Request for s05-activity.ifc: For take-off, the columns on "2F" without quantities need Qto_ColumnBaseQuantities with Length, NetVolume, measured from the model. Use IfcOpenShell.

First a look at what the model holds.

```python
import ifcopenshell
import ifcopenshell.util.element
import ifcopenshell.util.unit

model = ifcopenshell.open("s05-activity.ifc")
print(model.schema)
for unit_type in ("LENGTHUNIT", "AREAUNIT", "VOLUMEUNIT"):
    print(unit_type, ifcopenshell.util.unit.calculate_unit_scale(model, unit_type))
storey = next(s for s in model.by_type("IfcBuildingStorey") if s.Name == "2F")
columns = [e for e in ifcopenshell.util.element.get_decomposition(storey) if e.is_a("IfcColumn")]
for e in sorted(columns, key=lambda e: e.id()):
    print(e.id(), e.is_a(), e.Name, list(ifcopenshell.util.element.get_psets(e, qtos_only=True)), sep=" | ")
```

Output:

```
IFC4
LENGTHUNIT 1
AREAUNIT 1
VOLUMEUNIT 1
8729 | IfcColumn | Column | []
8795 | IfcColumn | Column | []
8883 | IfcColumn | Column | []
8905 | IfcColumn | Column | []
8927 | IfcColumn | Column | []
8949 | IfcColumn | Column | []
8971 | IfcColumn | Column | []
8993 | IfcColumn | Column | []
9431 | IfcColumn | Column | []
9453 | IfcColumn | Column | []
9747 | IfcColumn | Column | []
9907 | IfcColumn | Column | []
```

```python
import ifcopenshell
import ifcopenshell.api.pset
import ifcopenshell.geom
import ifcopenshell.util.element
import ifcopenshell.util.shape
import ifcopenshell.util.unit

model = ifcopenshell.open("s05-activity.ifc")
unit_scale = ifcopenshell.util.unit.calculate_unit_scale(model)
volume_scale = ifcopenshell.util.unit.calculate_unit_scale(model, "VOLUMEUNIT")
settings = ifcopenshell.geom.settings()

storey = next(s for s in model.by_type("IfcBuildingStorey") if s.Name == "2F")
columns = [e for e in ifcopenshell.util.element.get_decomposition(storey) if e.is_a("IfcColumn")]

for e in sorted(columns, key=lambda e: e.id()):
    if ifcopenshell.util.element.get_psets(e, qtos_only=True, should_inherit=False):
        continue
    # Geometry comes back in metres, in the element's own axes.
    shape = ifcopenshell.geom.create_shape(settings, e)
    values = {
        "Length": ifcopenshell.util.shape.get_z(shape.geometry) / unit_scale,
        "NetVolume": ifcopenshell.util.shape.get_volume(shape.geometry) / volume_scale,
    }
    qto = ifcopenshell.api.pset.add_qto(model, product=e, name="Qto_ColumnBaseQuantities")
    ifcopenshell.api.pset.edit_qto(model, qto=qto, properties=values)
    print(e.id(), {k: round(v, 3) for k, v in values.items()})

model.write("s05-activity_updated.ifc")
```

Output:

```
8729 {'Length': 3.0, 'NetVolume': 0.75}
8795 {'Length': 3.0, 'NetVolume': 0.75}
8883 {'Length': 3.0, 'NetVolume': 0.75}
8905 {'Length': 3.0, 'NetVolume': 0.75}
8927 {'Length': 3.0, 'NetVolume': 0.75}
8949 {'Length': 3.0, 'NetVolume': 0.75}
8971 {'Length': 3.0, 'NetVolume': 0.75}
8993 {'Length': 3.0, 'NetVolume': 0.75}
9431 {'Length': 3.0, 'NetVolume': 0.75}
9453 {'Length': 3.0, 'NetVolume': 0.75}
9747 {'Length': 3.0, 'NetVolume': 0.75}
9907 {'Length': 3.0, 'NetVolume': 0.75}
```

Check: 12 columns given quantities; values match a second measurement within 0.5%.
